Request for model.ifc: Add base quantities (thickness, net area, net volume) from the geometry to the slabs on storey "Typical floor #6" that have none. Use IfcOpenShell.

First a look at what the model holds.

```python
import ifcopenshell
import ifcopenshell.util.element
import ifcopenshell.util.unit

model = ifcopenshell.open("model.ifc")
print(model.schema)
for unit_type in ("LENGTHUNIT", "AREAUNIT", "VOLUMEUNIT"):
    print(unit_type, ifcopenshell.util.unit.calculate_unit_scale(model, unit_type))
storey = next(s for s in model.by_type("IfcBuildingStorey") if s.Name == "Typical floor #6")
slabs = [e for e in ifcopenshell.util.element.get_decomposition(storey) if e.is_a("IfcSlab")]
for e in sorted(slabs, key=lambda e: e.id()):
    print(e.id(), e.is_a(), e.Name, list(ifcopenshell.util.element.get_psets(e, qtos_only=True)), sep=" | ")
```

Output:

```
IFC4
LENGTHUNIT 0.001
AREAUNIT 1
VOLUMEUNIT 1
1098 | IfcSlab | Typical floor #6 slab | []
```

```python
import ifcopenshell
import ifcopenshell.api.pset
import ifcopenshell.geom
import ifcopenshell.util.element
import ifcopenshell.util.shape
import ifcopenshell.util.unit

model = ifcopenshell.open("model.ifc")
unit_scale = ifcopenshell.util.unit.calculate_unit_scale(model)
area_scale = ifcopenshell.util.unit.calculate_unit_scale(model, "AREAUNIT")
volume_scale = ifcopenshell.util.unit.calculate_unit_scale(model, "VOLUMEUNIT")
settings = ifcopenshell.geom.settings()

storey = next(s for s in model.by_type("IfcBuildingStorey") if s.Name == "Typical floor #6")
slabs = [e for e in ifcopenshell.util.element.get_decomposition(storey) if e.is_a("IfcSlab")]

for e in sorted(slabs, key=lambda e: e.id()):
    if ifcopenshell.util.element.get_psets(e, qtos_only=True, should_inherit=False):
        continue
    # Geometry comes back in metres, in the element's own axes.
    shape = ifcopenshell.geom.create_shape(settings, e)
    values = {
        "Width": ifcopenshell.util.shape.get_z(shape.geometry) / unit_scale,
        "NetArea": ifcopenshell.util.shape.get_footprint_area(shape.geometry) / area_scale,
        "NetVolume": ifcopenshell.util.shape.get_volume(shape.geometry) / volume_scale,
    }
    qto = ifcopenshell.api.pset.add_qto(model, product=e, name="Qto_SlabBaseQuantities")
    ifcopenshell.api.pset.edit_qto(model, qto=qto, properties=values)
    print(e.id(), {k: round(v, 3) for k, v in values.items()})

model.write("model_updated.ifc")
```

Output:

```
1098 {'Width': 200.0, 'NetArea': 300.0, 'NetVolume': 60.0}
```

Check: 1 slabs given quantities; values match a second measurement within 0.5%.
